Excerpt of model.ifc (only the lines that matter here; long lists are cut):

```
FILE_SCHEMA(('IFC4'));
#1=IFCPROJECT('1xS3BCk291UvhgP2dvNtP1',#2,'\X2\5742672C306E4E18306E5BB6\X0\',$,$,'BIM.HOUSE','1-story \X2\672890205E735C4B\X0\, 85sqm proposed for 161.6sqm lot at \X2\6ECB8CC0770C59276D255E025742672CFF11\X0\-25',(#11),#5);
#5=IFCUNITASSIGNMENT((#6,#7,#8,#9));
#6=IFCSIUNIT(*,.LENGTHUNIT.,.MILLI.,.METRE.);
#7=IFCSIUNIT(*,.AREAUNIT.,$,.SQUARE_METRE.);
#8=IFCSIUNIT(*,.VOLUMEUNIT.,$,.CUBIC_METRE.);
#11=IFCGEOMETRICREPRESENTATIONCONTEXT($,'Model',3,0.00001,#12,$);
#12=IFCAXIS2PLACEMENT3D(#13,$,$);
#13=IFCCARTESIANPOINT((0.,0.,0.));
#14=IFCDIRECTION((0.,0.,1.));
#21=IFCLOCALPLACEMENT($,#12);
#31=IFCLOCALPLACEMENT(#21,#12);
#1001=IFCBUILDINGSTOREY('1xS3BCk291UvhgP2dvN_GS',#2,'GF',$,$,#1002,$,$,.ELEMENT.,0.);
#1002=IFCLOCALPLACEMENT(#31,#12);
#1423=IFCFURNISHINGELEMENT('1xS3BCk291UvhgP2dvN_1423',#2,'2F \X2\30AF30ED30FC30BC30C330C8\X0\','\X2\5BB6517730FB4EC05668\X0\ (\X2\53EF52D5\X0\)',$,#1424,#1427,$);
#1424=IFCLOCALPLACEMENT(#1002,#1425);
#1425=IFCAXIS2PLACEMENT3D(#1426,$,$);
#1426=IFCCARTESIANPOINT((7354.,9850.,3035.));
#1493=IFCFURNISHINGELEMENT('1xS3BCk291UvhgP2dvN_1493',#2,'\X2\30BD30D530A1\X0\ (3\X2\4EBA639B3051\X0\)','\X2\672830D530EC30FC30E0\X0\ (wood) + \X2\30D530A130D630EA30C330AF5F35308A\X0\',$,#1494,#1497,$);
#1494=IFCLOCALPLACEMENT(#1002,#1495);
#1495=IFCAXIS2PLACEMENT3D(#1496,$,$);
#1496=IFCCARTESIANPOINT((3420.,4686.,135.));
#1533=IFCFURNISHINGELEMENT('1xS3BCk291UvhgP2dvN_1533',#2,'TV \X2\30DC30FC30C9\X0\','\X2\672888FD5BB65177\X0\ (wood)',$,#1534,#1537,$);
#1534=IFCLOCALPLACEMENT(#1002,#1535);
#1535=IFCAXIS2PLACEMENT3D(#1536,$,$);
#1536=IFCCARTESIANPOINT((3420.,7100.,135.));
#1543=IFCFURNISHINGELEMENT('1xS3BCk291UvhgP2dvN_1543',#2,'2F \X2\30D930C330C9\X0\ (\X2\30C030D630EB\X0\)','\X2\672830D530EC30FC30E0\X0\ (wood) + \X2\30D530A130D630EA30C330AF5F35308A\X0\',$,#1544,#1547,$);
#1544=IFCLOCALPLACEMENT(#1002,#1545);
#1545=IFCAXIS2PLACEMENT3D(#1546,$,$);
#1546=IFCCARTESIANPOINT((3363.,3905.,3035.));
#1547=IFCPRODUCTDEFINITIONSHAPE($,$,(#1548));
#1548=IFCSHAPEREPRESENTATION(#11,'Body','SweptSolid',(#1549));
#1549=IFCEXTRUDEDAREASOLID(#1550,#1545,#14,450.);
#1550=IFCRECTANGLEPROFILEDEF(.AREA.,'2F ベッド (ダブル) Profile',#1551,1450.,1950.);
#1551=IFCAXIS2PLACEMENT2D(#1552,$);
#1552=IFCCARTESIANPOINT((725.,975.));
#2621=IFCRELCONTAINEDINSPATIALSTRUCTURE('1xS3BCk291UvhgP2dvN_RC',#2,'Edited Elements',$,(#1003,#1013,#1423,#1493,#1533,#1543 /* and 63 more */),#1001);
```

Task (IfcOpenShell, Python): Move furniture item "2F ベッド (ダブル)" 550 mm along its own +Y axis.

```python
import ifcopenshell
import ifcopenshell.api.geometry
import ifcopenshell.util.placement

model = ifcopenshell.open("model.ifc")

item = model.by_guid("1xS3BCk291UvhgP2dvN_1543")
matrix = ifcopenshell.util.placement.get_local_placement(item.ObjectPlacement)
matrix[:3, 3] += matrix[:3, 1] * 550.0
ifcopenshell.api.geometry.edit_object_placement(model, product=item, matrix=matrix, is_si=False)

print(ifcopenshell.util.placement.get_local_placement(item.ObjectPlacement).round(3) + 0.0)

model.write("model_v2.ifc")
```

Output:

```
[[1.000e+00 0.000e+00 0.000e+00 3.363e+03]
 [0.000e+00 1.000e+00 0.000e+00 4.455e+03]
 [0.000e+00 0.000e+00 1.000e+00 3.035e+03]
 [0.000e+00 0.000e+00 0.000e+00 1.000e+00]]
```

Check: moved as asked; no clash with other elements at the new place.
